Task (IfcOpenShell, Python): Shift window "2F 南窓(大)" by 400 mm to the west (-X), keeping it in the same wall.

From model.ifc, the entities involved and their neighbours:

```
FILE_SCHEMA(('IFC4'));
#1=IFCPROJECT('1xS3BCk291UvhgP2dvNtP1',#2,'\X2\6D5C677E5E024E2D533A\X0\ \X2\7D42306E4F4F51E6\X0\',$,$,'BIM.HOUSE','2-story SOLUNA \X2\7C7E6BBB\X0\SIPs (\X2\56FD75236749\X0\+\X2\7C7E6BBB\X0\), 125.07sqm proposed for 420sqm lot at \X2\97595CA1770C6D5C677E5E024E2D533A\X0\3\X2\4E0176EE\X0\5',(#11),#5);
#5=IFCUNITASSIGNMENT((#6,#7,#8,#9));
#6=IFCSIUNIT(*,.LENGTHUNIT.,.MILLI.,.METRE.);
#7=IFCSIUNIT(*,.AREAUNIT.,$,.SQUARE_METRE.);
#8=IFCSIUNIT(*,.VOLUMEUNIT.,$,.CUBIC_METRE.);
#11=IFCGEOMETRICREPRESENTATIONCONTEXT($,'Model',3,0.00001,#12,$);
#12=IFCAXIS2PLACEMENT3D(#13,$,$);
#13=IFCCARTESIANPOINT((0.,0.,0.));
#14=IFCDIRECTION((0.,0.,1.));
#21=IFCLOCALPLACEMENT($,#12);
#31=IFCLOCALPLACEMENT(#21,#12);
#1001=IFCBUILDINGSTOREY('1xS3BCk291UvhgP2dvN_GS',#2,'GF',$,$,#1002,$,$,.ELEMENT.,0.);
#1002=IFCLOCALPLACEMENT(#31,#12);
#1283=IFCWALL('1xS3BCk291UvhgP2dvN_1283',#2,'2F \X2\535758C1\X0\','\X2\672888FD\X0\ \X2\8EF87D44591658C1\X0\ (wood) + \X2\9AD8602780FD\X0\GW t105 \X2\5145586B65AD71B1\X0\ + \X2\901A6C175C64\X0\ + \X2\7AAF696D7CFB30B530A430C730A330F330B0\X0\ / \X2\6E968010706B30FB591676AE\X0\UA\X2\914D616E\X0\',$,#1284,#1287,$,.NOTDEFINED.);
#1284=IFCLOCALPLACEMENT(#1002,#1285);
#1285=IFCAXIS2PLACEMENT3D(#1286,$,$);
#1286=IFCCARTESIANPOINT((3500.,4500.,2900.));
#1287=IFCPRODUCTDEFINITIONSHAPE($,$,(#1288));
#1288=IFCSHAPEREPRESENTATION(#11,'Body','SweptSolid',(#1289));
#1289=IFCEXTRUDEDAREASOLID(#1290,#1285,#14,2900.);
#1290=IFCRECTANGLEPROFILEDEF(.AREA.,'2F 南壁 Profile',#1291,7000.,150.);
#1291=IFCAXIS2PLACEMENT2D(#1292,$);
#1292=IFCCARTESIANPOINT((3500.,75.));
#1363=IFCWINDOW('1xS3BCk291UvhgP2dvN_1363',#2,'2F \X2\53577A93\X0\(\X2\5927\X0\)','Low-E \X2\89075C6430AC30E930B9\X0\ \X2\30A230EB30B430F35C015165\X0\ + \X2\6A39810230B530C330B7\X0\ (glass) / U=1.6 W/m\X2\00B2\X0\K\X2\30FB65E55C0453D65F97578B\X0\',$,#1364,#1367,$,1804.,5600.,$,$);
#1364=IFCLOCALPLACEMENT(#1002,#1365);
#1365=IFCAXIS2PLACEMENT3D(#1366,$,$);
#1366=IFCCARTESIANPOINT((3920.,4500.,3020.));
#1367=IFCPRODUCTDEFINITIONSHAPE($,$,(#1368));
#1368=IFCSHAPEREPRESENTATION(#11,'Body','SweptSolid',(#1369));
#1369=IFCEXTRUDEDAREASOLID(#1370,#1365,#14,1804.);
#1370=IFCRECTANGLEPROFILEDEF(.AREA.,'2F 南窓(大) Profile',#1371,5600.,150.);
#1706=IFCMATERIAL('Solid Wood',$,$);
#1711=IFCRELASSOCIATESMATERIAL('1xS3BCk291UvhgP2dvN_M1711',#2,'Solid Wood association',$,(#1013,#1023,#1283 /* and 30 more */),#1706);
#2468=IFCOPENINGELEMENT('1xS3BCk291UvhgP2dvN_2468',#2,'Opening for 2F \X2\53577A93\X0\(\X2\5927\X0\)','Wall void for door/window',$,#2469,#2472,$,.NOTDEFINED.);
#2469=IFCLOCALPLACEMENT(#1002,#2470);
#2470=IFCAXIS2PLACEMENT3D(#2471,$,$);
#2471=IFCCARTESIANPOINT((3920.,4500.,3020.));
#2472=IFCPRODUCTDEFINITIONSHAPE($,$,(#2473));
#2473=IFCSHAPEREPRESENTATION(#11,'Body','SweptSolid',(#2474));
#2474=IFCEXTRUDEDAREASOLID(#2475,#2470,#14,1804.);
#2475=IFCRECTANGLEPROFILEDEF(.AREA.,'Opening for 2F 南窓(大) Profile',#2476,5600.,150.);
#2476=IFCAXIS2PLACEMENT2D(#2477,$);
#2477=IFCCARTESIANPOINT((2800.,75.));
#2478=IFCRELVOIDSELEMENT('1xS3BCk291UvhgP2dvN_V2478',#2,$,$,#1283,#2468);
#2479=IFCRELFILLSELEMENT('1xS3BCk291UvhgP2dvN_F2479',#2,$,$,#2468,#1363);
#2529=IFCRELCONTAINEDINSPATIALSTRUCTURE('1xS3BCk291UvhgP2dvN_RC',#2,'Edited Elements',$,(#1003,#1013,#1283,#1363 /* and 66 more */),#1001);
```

```python
import ifcopenshell
import ifcopenshell.api.geometry
import ifcopenshell.util.placement
import ifcopenshell.util.unit

model = ifcopenshell.open("model.ifc")
unit_scale = ifcopenshell.util.unit.calculate_unit_scale(model)

window = model.by_guid("1xS3BCk291UvhgP2dvN_1363")
opening = window.FillsVoids[0].RelatingOpeningElement
wall = opening.VoidsElements[0].RelatingBuildingElement

wall_matrix = ifcopenshell.util.placement.get_local_placement(wall.ObjectPlacement)
shift = wall_matrix[:3, 0] * -0.4 / unit_scale
before = ifcopenshell.util.placement.get_local_placement(window.ObjectPlacement)[:3, 3].copy()

# The window is not placed relative to its opening, so move both.
for product in (opening, window):
    matrix = ifcopenshell.util.placement.get_local_placement(product.ObjectPlacement)
    matrix[:3, 3] += shift
    ifcopenshell.api.geometry.edit_object_placement(model, product=product, matrix=matrix, is_si=False)

after = ifcopenshell.util.placement.get_local_placement(window.ObjectPlacement)[:3, 3]
print("window moved by", (after - before).round(3) + 0.0)

model.write("model_updated.ifc")
```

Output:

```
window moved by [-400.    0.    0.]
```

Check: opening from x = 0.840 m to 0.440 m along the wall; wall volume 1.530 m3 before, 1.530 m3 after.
